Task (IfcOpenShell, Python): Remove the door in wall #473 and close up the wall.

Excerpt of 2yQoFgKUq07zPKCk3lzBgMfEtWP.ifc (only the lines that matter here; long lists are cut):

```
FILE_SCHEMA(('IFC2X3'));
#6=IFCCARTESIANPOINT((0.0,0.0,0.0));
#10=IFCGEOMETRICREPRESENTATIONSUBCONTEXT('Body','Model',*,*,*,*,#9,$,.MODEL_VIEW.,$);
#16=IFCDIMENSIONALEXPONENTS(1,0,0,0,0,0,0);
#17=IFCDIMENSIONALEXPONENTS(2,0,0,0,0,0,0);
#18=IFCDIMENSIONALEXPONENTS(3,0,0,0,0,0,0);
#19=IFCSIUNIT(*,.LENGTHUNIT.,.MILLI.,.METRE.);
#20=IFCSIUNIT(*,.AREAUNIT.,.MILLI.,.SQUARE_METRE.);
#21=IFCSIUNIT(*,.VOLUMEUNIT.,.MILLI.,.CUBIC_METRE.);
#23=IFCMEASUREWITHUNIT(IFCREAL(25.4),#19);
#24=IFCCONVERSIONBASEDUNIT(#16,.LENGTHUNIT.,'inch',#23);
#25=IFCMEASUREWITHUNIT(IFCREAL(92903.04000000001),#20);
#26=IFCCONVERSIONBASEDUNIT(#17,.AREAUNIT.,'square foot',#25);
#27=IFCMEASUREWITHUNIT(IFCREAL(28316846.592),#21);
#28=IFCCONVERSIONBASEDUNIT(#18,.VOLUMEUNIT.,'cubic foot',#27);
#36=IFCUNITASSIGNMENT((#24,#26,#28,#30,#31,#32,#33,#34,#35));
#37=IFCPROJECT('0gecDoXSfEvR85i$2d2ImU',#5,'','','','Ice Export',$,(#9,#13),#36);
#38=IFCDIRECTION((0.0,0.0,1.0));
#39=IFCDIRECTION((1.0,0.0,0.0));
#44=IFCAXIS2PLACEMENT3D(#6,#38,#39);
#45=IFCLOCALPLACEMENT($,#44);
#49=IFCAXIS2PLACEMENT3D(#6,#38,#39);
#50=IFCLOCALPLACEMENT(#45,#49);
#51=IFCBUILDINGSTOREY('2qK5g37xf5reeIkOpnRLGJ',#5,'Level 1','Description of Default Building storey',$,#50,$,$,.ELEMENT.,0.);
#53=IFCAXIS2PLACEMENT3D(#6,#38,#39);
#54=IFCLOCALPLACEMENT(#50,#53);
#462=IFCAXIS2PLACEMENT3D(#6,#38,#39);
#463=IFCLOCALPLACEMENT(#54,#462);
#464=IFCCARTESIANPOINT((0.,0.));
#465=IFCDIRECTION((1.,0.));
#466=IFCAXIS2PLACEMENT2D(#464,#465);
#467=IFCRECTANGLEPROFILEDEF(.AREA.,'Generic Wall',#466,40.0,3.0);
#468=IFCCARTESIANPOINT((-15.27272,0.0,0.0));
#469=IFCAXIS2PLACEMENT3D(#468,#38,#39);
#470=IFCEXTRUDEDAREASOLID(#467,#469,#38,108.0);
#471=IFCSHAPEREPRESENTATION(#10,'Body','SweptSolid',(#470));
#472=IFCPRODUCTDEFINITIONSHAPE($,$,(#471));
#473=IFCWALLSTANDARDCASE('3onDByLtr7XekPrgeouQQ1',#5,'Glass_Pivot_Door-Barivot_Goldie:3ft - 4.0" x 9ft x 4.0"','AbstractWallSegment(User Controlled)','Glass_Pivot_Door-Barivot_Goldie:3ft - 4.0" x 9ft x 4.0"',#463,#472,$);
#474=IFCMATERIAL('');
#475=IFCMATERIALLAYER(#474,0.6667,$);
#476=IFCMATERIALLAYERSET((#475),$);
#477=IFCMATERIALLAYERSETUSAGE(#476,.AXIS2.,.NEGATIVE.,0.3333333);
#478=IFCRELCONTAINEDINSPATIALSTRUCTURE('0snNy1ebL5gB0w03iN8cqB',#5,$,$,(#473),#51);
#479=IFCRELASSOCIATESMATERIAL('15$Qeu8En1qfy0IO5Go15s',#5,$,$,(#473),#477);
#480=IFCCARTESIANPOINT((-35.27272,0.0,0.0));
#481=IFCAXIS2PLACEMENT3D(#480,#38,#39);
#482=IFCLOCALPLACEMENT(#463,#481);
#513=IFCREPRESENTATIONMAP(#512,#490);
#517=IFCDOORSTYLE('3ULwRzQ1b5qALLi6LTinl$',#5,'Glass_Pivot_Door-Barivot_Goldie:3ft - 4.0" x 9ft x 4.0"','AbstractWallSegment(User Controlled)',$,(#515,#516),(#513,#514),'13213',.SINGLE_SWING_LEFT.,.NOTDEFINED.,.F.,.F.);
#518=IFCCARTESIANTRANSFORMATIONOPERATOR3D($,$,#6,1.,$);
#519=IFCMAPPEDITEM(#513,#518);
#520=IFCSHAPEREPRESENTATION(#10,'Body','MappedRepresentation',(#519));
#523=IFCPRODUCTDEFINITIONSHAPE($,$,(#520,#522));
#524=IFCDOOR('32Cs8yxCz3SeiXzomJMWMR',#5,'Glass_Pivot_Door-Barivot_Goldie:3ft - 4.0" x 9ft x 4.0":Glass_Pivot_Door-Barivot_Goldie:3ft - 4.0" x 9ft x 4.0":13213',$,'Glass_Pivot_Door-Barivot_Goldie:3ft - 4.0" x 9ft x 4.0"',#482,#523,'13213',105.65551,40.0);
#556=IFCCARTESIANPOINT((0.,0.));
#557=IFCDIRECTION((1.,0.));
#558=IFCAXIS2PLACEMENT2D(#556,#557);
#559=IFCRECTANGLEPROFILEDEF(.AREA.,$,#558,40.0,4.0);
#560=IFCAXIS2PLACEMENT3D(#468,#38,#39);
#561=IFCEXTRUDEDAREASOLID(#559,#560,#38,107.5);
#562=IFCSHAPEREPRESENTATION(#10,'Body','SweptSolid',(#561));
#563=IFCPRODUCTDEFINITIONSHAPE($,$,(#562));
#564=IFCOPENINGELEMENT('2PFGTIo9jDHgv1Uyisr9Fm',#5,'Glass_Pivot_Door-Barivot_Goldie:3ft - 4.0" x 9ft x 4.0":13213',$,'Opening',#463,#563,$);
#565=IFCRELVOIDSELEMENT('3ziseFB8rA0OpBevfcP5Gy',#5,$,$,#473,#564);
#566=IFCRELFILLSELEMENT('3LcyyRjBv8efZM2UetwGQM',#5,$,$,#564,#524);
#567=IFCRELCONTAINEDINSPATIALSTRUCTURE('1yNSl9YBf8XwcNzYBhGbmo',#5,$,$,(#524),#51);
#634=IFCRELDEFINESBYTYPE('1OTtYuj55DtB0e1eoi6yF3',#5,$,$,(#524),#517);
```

```python
import ifcopenshell
import ifcopenshell.api.feature
import ifcopenshell.api.root
import ifcopenshell.geom
import ifcopenshell.util.shape

model = ifcopenshell.open("2yQoFgKUq07zPKCk3lzBgMfEtWP.ifc")
settings = ifcopenshell.geom.settings()


def volume(element):
    """Net volume in cubic metres, openings subtracted."""
    shape = ifcopenshell.geom.create_shape(settings, element)
    return ifcopenshell.util.shape.get_volume(shape.geometry)


door = model.by_guid("32Cs8yxCz3SeiXzomJMWMR")
opening = door.FillsVoids[0].RelatingOpeningElement
wall = opening.VoidsElements[0].RelatingBuildingElement
before = volume(wall)

ifcopenshell.api.root.remove_product(model, product=door)
ifcopenshell.api.feature.remove_feature(model, feature=opening)

after = volume(wall)

print(f"wall volume {before:.3f} -> {after:.3f} m3")

model.write("2yQoFgKUq07zPKCk3lzBgMfEtWP_updated.ifc")
```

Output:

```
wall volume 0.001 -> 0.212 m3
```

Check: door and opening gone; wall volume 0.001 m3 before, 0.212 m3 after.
